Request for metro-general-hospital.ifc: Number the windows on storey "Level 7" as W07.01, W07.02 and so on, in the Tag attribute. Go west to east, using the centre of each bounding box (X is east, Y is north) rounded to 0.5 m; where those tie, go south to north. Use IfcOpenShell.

First a look at what the model holds.

```python
import ifcopenshell
import ifcopenshell.util.element
import ifcopenshell.util.placement

model = ifcopenshell.open("metro-general-hospital.ifc")
print(model.schema)
storey = next(s for s in model.by_type("IfcBuildingStorey") if s.Name == "Level 7")
windows = [e for e in ifcopenshell.util.element.get_decomposition(storey) if e.is_a("IfcWindow")]
for e in sorted(windows, key=lambda e: e.id()):
    origin = ifcopenshell.util.placement.get_local_placement(e.ObjectPlacement)[:3, 3]
    print(e.id(), e.Tag, e.Name, origin.round(2) + 0.0, sep=" | ")
```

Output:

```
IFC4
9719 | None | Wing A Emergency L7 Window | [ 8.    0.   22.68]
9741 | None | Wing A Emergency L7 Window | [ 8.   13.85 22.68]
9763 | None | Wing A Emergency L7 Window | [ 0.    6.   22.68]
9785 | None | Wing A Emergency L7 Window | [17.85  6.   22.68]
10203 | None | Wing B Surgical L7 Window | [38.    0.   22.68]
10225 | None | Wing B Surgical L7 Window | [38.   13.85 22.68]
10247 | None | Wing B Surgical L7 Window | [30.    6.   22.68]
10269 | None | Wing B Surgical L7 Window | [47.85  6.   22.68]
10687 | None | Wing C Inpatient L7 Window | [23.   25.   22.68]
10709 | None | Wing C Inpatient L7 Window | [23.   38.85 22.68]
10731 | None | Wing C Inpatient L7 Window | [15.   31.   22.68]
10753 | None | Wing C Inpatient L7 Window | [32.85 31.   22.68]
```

```python
import ifcopenshell
import ifcopenshell.geom
import ifcopenshell.util.element
import ifcopenshell.util.shape

model = ifcopenshell.open("metro-general-hospital.ifc")
settings = ifcopenshell.geom.settings()
settings.set("use-world-coords", True)


def centre(element):
    shape = ifcopenshell.geom.create_shape(settings, element)
    return ifcopenshell.util.shape.get_bbox_centroid(shape.geometry)


storey = next(s for s in model.by_type("IfcBuildingStorey") if s.Name == "Level 7")
windows = [e for e in ifcopenshell.util.element.get_decomposition(storey) if e.is_a("IfcWindow")]

# Insertion points can sit at a corner or the storey origin, so sort by the geometry (in metres).
centres = {e: centre(e) for e in windows}
windows.sort(key=lambda e: (round(centres[e][0] / 0.5), centres[e][1]))

for i, e in enumerate(windows, start=1):
    number = f"W07.{i:02d}"
    e.Tag = number
    print(e.id(), number)

model.write("metro-general-hospital_v2.ifc")
```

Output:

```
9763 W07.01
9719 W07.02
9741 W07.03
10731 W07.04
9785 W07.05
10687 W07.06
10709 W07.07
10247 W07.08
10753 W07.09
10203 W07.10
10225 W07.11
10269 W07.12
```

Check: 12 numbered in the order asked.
